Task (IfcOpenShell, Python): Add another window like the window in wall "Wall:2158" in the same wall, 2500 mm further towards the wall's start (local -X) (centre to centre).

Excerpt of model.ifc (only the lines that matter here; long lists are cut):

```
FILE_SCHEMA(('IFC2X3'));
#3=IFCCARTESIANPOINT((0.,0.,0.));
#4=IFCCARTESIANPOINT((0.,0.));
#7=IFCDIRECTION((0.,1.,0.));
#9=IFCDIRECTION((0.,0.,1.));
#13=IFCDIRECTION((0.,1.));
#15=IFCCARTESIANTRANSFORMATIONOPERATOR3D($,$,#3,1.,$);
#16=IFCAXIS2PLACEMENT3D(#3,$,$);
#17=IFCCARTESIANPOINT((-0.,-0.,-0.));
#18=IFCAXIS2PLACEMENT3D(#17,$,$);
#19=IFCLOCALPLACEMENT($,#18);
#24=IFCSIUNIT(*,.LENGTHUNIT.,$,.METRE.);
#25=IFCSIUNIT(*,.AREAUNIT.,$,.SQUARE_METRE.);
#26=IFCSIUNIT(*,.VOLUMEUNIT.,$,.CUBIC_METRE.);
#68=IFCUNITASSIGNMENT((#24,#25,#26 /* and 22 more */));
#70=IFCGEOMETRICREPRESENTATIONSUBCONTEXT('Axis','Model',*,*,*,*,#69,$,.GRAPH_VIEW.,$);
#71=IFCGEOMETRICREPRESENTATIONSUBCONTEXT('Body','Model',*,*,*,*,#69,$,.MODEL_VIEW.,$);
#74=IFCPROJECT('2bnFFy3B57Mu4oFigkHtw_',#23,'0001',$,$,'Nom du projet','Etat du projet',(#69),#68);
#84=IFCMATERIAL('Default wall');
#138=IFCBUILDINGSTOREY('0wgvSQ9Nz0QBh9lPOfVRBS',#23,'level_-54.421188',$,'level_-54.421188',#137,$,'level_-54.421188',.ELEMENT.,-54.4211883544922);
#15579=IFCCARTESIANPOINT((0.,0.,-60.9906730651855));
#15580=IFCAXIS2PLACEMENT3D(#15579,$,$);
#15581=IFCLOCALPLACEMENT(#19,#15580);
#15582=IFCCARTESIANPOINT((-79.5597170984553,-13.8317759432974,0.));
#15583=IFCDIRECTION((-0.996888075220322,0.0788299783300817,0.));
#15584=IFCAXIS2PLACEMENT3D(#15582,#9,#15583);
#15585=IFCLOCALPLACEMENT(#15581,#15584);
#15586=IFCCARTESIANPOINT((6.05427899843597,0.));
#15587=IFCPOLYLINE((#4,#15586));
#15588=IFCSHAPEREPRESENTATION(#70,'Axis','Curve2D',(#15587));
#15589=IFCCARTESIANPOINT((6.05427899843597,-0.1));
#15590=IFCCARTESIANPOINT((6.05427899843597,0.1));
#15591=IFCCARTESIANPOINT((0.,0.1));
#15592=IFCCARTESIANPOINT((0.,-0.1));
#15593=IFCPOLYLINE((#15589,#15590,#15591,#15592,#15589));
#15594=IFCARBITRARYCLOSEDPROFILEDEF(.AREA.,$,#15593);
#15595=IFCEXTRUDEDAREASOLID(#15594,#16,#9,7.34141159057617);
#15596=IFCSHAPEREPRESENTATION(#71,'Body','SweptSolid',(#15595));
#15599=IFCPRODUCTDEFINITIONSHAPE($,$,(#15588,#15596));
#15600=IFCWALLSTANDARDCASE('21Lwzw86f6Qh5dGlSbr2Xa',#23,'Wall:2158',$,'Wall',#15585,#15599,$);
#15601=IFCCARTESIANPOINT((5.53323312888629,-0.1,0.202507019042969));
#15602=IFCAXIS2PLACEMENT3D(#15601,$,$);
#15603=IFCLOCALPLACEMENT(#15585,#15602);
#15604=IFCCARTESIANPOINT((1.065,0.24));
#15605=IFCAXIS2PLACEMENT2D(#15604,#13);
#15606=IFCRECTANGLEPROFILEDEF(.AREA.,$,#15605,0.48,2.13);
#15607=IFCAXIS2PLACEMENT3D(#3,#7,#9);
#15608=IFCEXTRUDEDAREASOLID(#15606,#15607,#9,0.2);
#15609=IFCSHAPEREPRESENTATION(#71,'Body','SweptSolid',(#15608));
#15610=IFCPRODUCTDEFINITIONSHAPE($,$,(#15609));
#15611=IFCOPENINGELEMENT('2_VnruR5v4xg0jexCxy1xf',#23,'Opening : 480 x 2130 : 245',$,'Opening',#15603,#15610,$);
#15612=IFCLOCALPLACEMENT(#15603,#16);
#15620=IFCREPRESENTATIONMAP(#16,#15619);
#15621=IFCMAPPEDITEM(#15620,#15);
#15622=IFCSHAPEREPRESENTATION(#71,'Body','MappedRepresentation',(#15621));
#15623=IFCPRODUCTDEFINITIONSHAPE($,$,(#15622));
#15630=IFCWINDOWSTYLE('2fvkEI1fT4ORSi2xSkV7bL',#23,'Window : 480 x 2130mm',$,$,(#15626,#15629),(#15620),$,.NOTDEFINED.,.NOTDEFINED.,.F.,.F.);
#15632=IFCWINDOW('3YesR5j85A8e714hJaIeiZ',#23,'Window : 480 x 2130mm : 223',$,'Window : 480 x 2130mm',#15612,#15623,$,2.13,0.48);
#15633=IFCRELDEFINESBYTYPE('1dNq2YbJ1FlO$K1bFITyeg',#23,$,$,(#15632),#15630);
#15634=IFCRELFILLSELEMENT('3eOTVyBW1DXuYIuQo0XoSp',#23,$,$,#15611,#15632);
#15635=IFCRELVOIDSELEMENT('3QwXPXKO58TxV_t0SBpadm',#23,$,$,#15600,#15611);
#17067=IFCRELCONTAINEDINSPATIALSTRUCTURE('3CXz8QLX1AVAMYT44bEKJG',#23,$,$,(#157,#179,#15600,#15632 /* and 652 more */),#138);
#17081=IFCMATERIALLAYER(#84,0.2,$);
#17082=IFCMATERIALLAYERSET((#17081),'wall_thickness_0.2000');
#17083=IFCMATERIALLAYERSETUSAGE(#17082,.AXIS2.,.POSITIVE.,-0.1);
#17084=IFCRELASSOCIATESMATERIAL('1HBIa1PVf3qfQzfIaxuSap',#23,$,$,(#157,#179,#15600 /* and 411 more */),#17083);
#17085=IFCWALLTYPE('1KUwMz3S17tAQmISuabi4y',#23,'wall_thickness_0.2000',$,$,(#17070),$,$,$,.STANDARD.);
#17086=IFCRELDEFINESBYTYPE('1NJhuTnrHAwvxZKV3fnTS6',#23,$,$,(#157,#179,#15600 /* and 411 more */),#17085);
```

```python
import ifcopenshell
import ifcopenshell.api.feature
import ifcopenshell.api.geometry
import ifcopenshell.api.root
import ifcopenshell.geom
import ifcopenshell.util.element
import ifcopenshell.util.placement
import ifcopenshell.util.shape

model = ifcopenshell.open("model.ifc")
settings = ifcopenshell.geom.settings()


def volume(element):
    """Net volume in cubic metres, openings subtracted."""
    shape = ifcopenshell.geom.create_shape(settings, element)
    return ifcopenshell.util.shape.get_volume(shape.geometry)


window = model.by_guid("3YesR5j85A8e714hJaIeiZ")
opening = window.FillsVoids[0].RelatingOpeningElement
wall = opening.VoidsElements[0].RelatingBuildingElement
before = volume(wall)
shift = ifcopenshell.util.placement.get_local_placement(wall.ObjectPlacement)[:3, 0] * -2.5

# copy_class copies the void relationship, type, container and properties, but no geometry.
new_opening = ifcopenshell.api.root.copy_class(model, product=opening)
new_opening.Representation = ifcopenshell.util.element.copy_deep(
    model, opening.Representation, exclude=["IfcGeometricRepresentationContext", "IfcRepresentationMap"]
)
new_opening.Name = "Opening : 480 x 2130"
new_window = ifcopenshell.api.root.copy_class(model, product=window)
new_window.Representation = ifcopenshell.util.element.copy_deep(
    model, window.Representation, exclude=["IfcGeometricRepresentationContext", "IfcRepresentationMap"]
)
new_window.Name = "Window : 480 x 2130mm"
fills = ifcopenshell.api.feature.add_filling(model, opening=new_opening, element=new_window)
fills.OwnerHistory = new_window.OwnerHistory  # required in IFC2X3

for old, new in ((opening, new_opening), (window, new_window)):
    matrix = ifcopenshell.util.placement.get_local_placement(old.ObjectPlacement)
    matrix[:3, 3] += shift
    ifcopenshell.api.geometry.edit_object_placement(model, product=new, matrix=matrix, is_si=False)

after = volume(wall)

print(f"wall volume {before:.3f} -> {after:.3f} m3")

model.write("model_rev.ifc")
```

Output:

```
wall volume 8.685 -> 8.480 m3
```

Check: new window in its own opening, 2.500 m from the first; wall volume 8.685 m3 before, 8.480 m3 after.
